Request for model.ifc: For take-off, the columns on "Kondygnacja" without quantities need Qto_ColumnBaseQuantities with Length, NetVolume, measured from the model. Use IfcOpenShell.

First a look at what the model holds.

```python
import ifcopenshell
import ifcopenshell.util.element
import ifcopenshell.util.unit

model = ifcopenshell.open("model.ifc")
print(model.schema)
for unit_type in ("LENGTHUNIT", "AREAUNIT", "VOLUMEUNIT"):
    print(unit_type, ifcopenshell.util.unit.calculate_unit_scale(model, unit_type))
storey = next(s for s in model.by_type("IfcBuildingStorey") if s.Name == "Kondygnacja")
columns = [e for e in ifcopenshell.util.element.get_decomposition(storey) if e.is_a("IfcColumn")]
for e in sorted(columns, key=lambda e: e.id()):
    print(e.id(), e.is_a(), e.Name, list(ifcopenshell.util.element.get_psets(e, qtos_only=True)), sep=" | ")
```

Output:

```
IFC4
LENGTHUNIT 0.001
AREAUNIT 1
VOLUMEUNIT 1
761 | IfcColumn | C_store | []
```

```python
import ifcopenshell
import ifcopenshell.api.pset
import ifcopenshell.geom
import ifcopenshell.util.element
import ifcopenshell.util.shape
import ifcopenshell.util.unit

model = ifcopenshell.open("model.ifc")
unit_scale = ifcopenshell.util.unit.calculate_unit_scale(model)
volume_scale = ifcopenshell.util.unit.calculate_unit_scale(model, "VOLUMEUNIT")
settings = ifcopenshell.geom.settings()

storey = next(s for s in model.by_type("IfcBuildingStorey") if s.Name == "Kondygnacja")
columns = [e for e in ifcopenshell.util.element.get_decomposition(storey) if e.is_a("IfcColumn")]

for e in sorted(columns, key=lambda e: e.id()):
    if ifcopenshell.util.element.get_psets(e, qtos_only=True, should_inherit=False):
        continue
    # Geometry comes back in metres, in the element's own axes.
    shape = ifcopenshell.geom.create_shape(settings, e)
    values = {
        "Length": ifcopenshell.util.shape.get_z(shape.geometry) / unit_scale,
        "NetVolume": ifcopenshell.util.shape.get_volume(shape.geometry) / volume_scale,
    }
    qto = ifcopenshell.api.pset.add_qto(model, product=e, name="Qto_ColumnBaseQuantities")
    ifcopenshell.api.pset.edit_qto(model, qto=qto, properties=values)
    print(e.id(), {k: round(v, 3) for k, v in values.items()})

model.write("model_updated.ifc")
```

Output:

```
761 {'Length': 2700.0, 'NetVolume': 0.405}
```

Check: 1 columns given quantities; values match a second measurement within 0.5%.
